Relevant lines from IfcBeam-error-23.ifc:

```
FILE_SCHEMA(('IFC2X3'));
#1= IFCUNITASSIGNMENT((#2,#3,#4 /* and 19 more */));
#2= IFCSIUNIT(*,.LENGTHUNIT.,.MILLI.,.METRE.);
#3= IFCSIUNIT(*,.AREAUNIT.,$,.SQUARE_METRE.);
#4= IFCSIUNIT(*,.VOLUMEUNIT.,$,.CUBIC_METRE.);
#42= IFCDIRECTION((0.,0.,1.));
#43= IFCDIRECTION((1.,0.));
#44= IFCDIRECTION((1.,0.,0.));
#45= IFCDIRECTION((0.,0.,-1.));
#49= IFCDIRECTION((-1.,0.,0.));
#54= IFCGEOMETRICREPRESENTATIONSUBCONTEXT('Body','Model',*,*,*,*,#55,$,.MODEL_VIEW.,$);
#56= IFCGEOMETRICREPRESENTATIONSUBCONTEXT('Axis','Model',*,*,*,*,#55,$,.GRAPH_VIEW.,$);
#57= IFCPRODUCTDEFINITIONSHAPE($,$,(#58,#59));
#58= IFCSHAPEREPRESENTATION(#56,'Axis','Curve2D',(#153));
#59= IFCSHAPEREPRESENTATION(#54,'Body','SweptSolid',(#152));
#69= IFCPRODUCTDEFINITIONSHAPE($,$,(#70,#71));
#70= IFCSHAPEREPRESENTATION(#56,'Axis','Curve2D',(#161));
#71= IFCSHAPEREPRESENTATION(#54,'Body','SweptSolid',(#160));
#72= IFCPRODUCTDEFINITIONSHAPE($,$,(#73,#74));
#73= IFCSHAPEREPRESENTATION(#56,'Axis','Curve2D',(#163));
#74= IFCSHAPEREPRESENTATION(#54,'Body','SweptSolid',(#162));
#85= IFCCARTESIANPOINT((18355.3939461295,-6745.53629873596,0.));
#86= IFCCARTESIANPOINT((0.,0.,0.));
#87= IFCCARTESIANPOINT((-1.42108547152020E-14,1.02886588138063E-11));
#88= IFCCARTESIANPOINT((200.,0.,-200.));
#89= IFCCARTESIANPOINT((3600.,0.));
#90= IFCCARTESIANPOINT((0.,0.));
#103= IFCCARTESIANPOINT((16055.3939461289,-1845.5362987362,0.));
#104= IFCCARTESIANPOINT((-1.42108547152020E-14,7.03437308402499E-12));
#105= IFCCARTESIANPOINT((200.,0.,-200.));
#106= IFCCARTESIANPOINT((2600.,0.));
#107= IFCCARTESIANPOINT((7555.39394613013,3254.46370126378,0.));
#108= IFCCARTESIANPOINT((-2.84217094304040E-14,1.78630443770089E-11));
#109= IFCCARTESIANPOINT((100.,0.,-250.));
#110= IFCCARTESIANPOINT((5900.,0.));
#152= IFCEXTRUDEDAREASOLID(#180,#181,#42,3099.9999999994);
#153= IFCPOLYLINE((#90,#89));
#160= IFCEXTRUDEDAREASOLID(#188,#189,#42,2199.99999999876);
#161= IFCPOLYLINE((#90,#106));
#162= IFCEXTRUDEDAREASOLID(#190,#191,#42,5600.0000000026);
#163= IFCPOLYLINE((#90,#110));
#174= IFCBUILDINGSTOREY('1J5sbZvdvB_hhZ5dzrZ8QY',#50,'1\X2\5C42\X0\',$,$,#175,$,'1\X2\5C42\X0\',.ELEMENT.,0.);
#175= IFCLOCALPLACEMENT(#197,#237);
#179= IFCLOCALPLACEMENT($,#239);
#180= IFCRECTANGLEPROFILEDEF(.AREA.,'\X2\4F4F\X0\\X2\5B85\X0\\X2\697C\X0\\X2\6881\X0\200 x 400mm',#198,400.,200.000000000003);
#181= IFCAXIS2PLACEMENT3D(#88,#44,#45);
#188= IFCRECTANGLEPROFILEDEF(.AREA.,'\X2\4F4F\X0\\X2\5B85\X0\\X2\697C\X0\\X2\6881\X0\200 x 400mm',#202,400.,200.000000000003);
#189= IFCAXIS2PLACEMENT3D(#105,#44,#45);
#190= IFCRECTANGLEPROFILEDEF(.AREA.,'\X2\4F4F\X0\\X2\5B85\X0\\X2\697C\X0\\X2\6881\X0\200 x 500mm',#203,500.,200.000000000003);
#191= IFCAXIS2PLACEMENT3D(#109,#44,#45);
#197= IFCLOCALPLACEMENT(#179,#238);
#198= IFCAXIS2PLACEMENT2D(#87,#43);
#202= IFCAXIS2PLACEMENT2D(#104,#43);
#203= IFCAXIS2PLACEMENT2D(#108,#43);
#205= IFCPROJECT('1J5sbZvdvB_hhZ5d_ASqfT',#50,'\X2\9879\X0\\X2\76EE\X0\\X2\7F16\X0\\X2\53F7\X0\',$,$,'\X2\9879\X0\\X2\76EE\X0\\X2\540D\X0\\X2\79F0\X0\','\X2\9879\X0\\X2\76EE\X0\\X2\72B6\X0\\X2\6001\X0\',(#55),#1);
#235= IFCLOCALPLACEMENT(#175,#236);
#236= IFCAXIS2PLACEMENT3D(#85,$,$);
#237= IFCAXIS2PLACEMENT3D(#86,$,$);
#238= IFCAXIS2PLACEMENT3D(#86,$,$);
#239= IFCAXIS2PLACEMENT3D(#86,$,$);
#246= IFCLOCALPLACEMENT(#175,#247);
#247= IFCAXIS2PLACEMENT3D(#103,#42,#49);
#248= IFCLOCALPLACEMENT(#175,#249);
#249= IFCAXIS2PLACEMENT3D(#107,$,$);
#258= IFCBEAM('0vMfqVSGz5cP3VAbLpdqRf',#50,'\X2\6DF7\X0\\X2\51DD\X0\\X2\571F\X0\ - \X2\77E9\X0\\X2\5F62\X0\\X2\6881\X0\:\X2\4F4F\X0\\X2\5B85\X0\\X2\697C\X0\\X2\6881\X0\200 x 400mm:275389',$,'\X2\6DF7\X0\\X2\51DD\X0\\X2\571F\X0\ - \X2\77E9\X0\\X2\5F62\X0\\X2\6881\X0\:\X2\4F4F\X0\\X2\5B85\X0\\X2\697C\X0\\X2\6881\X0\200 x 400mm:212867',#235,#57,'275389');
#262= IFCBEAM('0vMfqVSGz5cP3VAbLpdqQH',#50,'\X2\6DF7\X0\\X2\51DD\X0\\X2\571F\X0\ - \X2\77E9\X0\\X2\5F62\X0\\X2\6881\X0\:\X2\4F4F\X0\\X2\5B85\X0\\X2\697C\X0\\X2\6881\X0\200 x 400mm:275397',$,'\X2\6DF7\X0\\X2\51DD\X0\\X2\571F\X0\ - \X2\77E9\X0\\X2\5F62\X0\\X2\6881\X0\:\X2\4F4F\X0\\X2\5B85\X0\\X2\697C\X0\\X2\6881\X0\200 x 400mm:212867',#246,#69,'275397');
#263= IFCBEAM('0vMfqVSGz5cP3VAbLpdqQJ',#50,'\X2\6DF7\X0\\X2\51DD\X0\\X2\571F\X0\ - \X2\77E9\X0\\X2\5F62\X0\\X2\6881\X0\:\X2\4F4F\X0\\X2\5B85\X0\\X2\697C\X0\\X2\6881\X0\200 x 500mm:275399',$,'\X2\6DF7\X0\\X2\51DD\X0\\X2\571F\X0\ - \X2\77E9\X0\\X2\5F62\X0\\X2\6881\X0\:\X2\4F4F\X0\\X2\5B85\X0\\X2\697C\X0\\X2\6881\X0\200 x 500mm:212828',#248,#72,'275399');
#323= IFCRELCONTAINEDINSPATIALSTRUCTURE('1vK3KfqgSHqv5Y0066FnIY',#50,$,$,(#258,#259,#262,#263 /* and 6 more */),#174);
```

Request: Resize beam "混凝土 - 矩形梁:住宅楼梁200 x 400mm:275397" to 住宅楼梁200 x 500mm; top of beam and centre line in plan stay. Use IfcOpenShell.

```python
import ifcopenshell
import ifcopenshell.util.element
import ifcopenshell.util.representation

model = ifcopenshell.open("IfcBeam-error-23.ifc")

member = model.by_guid("0vMfqVSGz5cP3VAbLpdqQH")
source = next(p for p in model.by_type("IfcRectangleProfileDef") if p.ProfileName == "住宅楼梁200 x 500mm")

body = ifcopenshell.util.representation.get_representation(member, "Model", "Body")
solid = body.Items[0]
old_profile = solid.SweptArea

# Copy the section's sizes but keep this member's own profile position.
profile = ifcopenshell.util.element.copy(model, source)
# Profiles are centred, so shift by half the change in depth to hold the top.
shift = (old_profile.XDim - profile.XDim) / 2
x, y = old_profile.Position.Location.Coordinates
up = (-1.0, 0.0)  # upwards, in the solid's own plane
location = model.createIfcCartesianPoint((x + up[0] * shift, y + up[1] * shift))
profile.Position = model.createIfcAxis2Placement2D(location, old_profile.Position.RefDirection)
solid.SweptArea = profile
if not model.get_total_inverses(old_profile):
    ifcopenshell.util.element.remove_deep2(model, old_profile)
member.Name = member.Name.replace("住宅楼梁200 x 400mm", "住宅楼梁200 x 500mm")
member.ObjectType = member.ObjectType.replace("住宅楼梁200 x 400mm", "住宅楼梁200 x 500mm")

print(solid.SweptArea)

model.write("IfcBeam-error-23-out.ifc")
```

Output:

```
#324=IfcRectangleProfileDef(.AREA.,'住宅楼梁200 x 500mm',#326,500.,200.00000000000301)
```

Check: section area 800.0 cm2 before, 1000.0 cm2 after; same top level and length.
